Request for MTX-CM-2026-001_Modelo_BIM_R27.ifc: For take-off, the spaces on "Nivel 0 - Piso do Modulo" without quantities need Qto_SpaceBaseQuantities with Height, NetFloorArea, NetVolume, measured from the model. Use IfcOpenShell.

First a look at what the model holds.

```python
import ifcopenshell
import ifcopenshell.util.element
import ifcopenshell.util.unit

model = ifcopenshell.open("MTX-CM-2026-001_Modelo_BIM_R27.ifc")
print(model.schema)
for unit_type in ("LENGTHUNIT", "AREAUNIT", "VOLUMEUNIT"):
    print(unit_type, ifcopenshell.util.unit.calculate_unit_scale(model, unit_type))
storey = next(s for s in model.by_type("IfcBuildingStorey") if s.Name == "Nivel 0 - Piso do Modulo")
spaces = [e for e in ifcopenshell.util.element.get_decomposition(storey) if e.is_a("IfcSpace")]
for e in sorted(spaces, key=lambda e: e.id()):
    print(e.id(), e.is_a(), e.Name, list(ifcopenshell.util.element.get_psets(e, qtos_only=True)), sep=" | ")
```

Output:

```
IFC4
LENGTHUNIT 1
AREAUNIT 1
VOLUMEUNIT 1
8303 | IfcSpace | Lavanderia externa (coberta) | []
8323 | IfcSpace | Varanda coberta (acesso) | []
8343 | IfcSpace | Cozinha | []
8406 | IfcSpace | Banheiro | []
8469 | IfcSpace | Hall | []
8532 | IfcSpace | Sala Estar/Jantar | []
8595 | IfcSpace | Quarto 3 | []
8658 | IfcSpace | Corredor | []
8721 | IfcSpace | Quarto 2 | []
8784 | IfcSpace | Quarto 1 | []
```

```python
import ifcopenshell
import ifcopenshell.api.pset
import ifcopenshell.geom
import ifcopenshell.util.element
import ifcopenshell.util.shape
import ifcopenshell.util.unit

model = ifcopenshell.open("MTX-CM-2026-001_Modelo_BIM_R27.ifc")
unit_scale = ifcopenshell.util.unit.calculate_unit_scale(model)
area_scale = ifcopenshell.util.unit.calculate_unit_scale(model, "AREAUNIT")
volume_scale = ifcopenshell.util.unit.calculate_unit_scale(model, "VOLUMEUNIT")
settings = ifcopenshell.geom.settings()

storey = next(s for s in model.by_type("IfcBuildingStorey") if s.Name == "Nivel 0 - Piso do Modulo")
spaces = [e for e in ifcopenshell.util.element.get_decomposition(storey) if e.is_a("IfcSpace")]

for e in sorted(spaces, key=lambda e: e.id()):
    if ifcopenshell.util.element.get_psets(e, qtos_only=True, should_inherit=False):
        continue
    # Geometry comes back in metres, in the element's own axes.
    shape = ifcopenshell.geom.create_shape(settings, e)
    values = {
        "Height": ifcopenshell.util.shape.get_z(shape.geometry) / unit_scale,
        "NetFloorArea": ifcopenshell.util.shape.get_footprint_area(shape.geometry) / area_scale,
        "NetVolume": ifcopenshell.util.shape.get_volume(shape.geometry) / volume_scale,
    }
    qto = ifcopenshell.api.pset.add_qto(model, product=e, name="Qto_SpaceBaseQuantities")
    ifcopenshell.api.pset.edit_qto(model, qto=qto, properties=values)
    print(e.id(), {k: round(v, 3) for k, v in values.items()})

model.write("MTX-CM-2026-001_Modelo_BIM_R27_v2.ifc")
```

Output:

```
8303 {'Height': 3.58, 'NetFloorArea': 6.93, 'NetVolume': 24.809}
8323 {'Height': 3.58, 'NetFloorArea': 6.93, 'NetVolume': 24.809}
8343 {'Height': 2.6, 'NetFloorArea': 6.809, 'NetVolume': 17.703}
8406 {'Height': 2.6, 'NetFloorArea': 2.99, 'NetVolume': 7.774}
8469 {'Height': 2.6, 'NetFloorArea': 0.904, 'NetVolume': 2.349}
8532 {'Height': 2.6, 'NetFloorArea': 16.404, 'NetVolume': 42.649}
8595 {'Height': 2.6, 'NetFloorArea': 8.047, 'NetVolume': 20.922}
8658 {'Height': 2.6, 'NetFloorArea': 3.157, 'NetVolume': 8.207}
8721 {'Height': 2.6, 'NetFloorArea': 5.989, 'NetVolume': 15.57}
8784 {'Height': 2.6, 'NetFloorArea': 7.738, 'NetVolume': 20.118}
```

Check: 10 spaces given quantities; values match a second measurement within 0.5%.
